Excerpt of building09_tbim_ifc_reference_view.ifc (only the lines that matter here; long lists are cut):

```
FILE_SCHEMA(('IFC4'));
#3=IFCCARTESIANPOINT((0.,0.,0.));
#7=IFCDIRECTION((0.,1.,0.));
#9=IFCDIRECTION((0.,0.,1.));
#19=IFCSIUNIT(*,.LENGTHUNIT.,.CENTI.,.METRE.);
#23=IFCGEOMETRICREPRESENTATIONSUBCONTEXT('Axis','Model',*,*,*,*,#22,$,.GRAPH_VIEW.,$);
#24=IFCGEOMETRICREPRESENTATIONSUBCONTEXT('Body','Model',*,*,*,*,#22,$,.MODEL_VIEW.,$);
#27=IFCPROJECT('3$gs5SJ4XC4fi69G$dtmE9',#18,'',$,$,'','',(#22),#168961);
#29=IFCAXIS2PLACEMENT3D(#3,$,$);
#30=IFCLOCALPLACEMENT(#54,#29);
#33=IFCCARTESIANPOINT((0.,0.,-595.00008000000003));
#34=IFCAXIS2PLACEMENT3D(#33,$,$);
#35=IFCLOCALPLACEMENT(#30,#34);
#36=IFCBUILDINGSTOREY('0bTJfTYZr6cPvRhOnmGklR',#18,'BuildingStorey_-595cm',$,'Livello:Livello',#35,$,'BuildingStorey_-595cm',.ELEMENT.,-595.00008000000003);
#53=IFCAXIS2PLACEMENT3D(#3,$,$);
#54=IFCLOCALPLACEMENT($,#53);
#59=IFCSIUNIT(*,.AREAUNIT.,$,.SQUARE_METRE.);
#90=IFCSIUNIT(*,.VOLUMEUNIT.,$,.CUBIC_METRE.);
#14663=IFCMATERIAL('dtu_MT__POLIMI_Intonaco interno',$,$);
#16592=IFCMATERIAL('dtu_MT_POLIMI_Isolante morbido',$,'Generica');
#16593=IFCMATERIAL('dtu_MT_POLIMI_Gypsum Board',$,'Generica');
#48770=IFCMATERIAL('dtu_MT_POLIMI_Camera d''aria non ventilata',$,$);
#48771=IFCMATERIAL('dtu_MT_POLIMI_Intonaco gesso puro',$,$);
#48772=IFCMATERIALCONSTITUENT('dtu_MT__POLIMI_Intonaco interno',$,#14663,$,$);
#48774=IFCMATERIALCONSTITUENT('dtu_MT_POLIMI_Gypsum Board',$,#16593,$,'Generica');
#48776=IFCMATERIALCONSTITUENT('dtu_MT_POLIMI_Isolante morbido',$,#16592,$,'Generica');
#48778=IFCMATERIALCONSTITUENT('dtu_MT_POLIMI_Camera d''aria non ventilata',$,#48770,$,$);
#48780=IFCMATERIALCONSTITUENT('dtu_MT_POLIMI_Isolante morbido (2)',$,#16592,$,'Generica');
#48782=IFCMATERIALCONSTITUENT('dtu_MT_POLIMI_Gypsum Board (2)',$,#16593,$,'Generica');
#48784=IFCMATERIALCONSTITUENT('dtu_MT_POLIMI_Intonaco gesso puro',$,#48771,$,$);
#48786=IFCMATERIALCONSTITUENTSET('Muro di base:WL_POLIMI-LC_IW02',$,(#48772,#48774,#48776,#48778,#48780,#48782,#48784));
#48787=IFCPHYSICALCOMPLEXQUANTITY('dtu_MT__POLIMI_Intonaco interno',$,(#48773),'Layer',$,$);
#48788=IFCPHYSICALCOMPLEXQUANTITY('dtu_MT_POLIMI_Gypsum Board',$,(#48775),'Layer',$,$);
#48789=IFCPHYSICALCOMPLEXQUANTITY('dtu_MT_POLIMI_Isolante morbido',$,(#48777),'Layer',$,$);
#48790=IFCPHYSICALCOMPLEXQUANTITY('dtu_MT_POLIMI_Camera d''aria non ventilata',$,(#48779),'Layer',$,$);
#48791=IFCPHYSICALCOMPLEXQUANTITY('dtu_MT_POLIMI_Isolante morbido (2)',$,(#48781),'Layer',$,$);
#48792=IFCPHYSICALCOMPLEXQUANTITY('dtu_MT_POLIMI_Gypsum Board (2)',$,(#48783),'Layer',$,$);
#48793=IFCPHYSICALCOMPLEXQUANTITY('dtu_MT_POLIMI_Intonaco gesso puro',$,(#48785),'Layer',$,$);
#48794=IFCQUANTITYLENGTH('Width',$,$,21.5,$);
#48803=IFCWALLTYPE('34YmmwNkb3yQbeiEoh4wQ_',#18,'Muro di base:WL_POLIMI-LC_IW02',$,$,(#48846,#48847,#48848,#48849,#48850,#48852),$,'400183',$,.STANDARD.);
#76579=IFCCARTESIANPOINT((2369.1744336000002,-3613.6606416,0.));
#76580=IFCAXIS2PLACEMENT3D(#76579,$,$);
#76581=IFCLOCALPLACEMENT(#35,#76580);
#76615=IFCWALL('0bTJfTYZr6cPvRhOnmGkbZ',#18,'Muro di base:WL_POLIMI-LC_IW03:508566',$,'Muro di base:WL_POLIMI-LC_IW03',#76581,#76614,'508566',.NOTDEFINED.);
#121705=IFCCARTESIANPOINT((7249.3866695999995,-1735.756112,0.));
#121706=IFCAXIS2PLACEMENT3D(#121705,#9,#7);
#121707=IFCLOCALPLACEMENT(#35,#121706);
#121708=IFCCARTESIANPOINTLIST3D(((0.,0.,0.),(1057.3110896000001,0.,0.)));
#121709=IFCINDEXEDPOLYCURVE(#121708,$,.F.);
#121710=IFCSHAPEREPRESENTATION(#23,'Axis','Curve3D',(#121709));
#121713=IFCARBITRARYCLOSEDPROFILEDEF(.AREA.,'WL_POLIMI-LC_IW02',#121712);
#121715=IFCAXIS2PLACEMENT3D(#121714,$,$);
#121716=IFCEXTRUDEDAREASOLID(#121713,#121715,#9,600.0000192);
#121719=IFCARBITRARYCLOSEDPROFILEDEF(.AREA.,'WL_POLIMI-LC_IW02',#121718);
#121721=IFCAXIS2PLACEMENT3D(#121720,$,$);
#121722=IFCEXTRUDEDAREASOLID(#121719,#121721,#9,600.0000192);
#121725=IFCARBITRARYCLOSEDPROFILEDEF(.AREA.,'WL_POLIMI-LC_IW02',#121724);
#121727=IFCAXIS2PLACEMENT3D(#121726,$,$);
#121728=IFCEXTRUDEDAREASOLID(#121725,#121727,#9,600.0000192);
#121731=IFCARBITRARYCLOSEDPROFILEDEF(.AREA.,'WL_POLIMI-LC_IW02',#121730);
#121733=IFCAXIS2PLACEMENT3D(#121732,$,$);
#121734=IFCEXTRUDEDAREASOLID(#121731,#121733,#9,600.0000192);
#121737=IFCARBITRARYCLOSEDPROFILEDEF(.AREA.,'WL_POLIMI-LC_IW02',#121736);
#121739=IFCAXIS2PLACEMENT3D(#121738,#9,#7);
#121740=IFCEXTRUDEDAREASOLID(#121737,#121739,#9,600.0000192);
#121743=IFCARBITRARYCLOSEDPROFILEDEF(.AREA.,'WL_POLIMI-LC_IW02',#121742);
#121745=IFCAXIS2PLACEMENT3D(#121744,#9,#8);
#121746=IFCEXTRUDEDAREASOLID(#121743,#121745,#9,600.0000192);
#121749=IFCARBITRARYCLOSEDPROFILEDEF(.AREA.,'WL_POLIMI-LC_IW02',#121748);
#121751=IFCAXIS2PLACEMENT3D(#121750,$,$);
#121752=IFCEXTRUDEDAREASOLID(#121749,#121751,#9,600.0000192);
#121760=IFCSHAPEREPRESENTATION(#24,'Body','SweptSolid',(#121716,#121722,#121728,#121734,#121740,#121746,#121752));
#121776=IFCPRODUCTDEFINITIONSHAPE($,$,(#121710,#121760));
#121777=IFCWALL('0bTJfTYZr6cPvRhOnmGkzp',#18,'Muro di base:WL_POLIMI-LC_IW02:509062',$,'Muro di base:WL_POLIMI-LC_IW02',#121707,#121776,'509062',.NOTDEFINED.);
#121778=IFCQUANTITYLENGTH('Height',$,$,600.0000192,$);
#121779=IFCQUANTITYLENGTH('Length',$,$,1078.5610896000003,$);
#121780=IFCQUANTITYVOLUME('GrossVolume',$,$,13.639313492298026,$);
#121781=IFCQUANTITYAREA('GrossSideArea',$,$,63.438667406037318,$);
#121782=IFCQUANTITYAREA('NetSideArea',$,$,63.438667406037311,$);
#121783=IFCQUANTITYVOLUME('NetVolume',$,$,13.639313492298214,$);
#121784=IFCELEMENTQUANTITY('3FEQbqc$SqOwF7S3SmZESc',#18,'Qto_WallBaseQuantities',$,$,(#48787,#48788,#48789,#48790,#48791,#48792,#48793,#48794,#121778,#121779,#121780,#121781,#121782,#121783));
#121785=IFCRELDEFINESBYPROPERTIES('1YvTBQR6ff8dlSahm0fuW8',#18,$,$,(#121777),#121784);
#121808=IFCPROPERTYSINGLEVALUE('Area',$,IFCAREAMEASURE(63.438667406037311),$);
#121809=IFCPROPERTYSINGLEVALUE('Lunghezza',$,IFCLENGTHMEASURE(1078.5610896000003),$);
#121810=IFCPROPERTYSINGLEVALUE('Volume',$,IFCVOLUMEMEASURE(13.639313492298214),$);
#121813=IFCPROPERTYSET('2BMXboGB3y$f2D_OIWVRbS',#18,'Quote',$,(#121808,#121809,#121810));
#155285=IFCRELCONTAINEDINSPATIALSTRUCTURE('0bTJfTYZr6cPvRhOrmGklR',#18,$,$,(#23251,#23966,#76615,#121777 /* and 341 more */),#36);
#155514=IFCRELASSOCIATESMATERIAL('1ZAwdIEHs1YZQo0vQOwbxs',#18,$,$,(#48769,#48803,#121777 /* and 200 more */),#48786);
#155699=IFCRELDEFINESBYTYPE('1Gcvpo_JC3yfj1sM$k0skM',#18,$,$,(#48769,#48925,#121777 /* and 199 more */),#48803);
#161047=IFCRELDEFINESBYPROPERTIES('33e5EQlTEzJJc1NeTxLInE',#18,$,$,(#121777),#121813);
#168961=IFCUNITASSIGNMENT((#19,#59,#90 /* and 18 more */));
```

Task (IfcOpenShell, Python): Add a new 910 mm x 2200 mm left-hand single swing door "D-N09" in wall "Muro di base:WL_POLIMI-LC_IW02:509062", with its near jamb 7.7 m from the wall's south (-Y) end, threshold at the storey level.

```python
import numpy as np
import ifcopenshell
import ifcopenshell.api.feature
import ifcopenshell.api.geometry
import ifcopenshell.api.pset
import ifcopenshell.api.root
import ifcopenshell.api.spatial
import ifcopenshell.geom
import ifcopenshell.util.element
import ifcopenshell.util.placement
import ifcopenshell.util.representation
import ifcopenshell.util.shape
import ifcopenshell.util.unit

model = ifcopenshell.open("building09_tbim_ifc_reference_view.ifc")
unit_scale = ifcopenshell.util.unit.calculate_unit_scale(model)
area_scale = ifcopenshell.util.unit.calculate_unit_scale(model, "AREAUNIT")
volume_scale = ifcopenshell.util.unit.calculate_unit_scale(model, "VOLUMEUNIT")
settings = ifcopenshell.geom.settings()


def volume(element):
    """Net volume in cubic metres, openings subtracted."""
    shape = ifcopenshell.geom.create_shape(settings, element)
    return ifcopenshell.util.shape.get_volume(shape.geometry)


wall = model.by_id(121777)
storey = ifcopenshell.util.element.get_container(wall, ifc_class="IfcBuildingStorey")
context = ifcopenshell.util.representation.get_context(model, "Model", "Body", "MODEL_VIEW")
before = volume(wall)

width, height, from_end, sill = 0.91, 2.2, 7.7, 0.0  # metres

# The wall runs along its own X axis, and the end named is its -X end.
wall_shape = ifcopenshell.geom.create_shape(settings, wall)
x, y, z = ifcopenshell.util.shape.get_vertices(wall_shape.geometry).T
start = x.min() + from_end
face, thickness = float(y.min()), float(y.max() - y.min())
wall_matrix = ifcopenshell.util.placement.get_local_placement(wall.ObjectPlacement)
level = ifcopenshell.util.placement.get_local_placement(storey.ObjectPlacement)[2, 3]


def in_wall(x, y):
    """Placement at x, y metres in the wall's axes, at sill height."""
    matrix = wall_matrix.copy()
    matrix[:, 3] = wall_matrix @ np.array([x / unit_scale, y / unit_scale, 0.0, 1.0])
    matrix[2, 3] = level + sill / unit_scale
    return matrix


# Opening: a box that overshoots both wall faces by 50 mm.
opening = ifcopenshell.api.root.create_entity(model, ifc_class="IfcOpeningElement", predefined_type="OPENING")
box = ifcopenshell.api.geometry.add_wall_representation(
    model, context=context, length=width, height=height, thickness=thickness + 0.1
)
ifcopenshell.api.geometry.assign_representation(model, product=opening, representation=box)
ifcopenshell.api.geometry.edit_object_placement(model, product=opening, matrix=in_wall(start, face - 0.05), is_si=False)
ifcopenshell.api.feature.add_feature(model, feature=opening, element=wall)

door = ifcopenshell.api.root.create_entity(model, ifc_class="IfcDoor", name="D-N09", predefined_type="DOOR")
door.OverallWidth, door.OverallHeight = width / unit_scale, height / unit_scale
door.OperationType = "SINGLE_SWING_LEFT"
body = ifcopenshell.api.geometry.add_door_representation(
    model,
    context=context,
    overall_width=door.OverallWidth,
    overall_height=door.OverallHeight,
    operation_type="SINGLE_SWING_LEFT",
    lining_properties={"LiningDepth": thickness / unit_scale, "ThresholdDepth": thickness / unit_scale},
)
ifcopenshell.api.geometry.assign_representation(model, product=door, representation=body)
ifcopenshell.api.spatial.assign_container(model, products=[door], relating_structure=storey)
ifcopenshell.api.feature.add_filling(model, opening=opening, element=door)

# The lining spans the wall, so the door starts at the wall face.
ifcopenshell.api.geometry.edit_object_placement(model, product=door, matrix=in_wall(start, face), is_si=False)

after = volume(wall)

# Update the wall's stored quantities.
qto = model.by_id(ifcopenshell.util.element.get_pset(wall, "Qto_WallBaseQuantities", should_inherit=False)["id"])
ifcopenshell.api.pset.edit_qto(model, qto=qto, properties={
    "NetSideArea": after / thickness / area_scale,
    "NetVolume": after / volume_scale,
})
pset = model.by_id(ifcopenshell.util.element.get_pset(wall, "Quote", should_inherit=False)["id"])
ifcopenshell.api.pset.edit_pset(model, pset=pset, properties={
    "Area": model.create_entity("IfcAreaMeasure", after / thickness / area_scale),
    "Volume": model.create_entity("IfcVolumeMeasure", after / volume_scale),
})

print(f"wall volume {before:.3f} -> {after:.3f} m3")

model.write("building09_tbim_ifc_reference_view_rev.ifc")
```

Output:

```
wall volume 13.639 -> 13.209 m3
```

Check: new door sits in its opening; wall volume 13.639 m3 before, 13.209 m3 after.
